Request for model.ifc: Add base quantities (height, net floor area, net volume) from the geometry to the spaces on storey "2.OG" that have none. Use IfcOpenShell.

First a look at what the model holds.

```python
import ifcopenshell
import ifcopenshell.util.element
import ifcopenshell.util.unit

model = ifcopenshell.open("model.ifc")
print(model.schema)
for unit_type in ("LENGTHUNIT", "AREAUNIT", "VOLUMEUNIT"):
    print(unit_type, ifcopenshell.util.unit.calculate_unit_scale(model, unit_type))
storey = next(s for s in model.by_type("IfcBuildingStorey") if s.Name == "2.OG")
spaces = [e for e in ifcopenshell.util.element.get_decomposition(storey) if e.is_a("IfcSpace")]
for e in sorted(spaces, key=lambda e: e.id()):
    print(e.id(), e.is_a(), e.Name, list(ifcopenshell.util.element.get_psets(e, qtos_only=True)), sep=" | ")
```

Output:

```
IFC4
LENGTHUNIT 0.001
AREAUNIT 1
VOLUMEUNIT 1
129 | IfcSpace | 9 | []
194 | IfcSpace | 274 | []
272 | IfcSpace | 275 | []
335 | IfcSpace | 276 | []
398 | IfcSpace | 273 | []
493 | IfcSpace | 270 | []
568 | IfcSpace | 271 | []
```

```python
import ifcopenshell
import ifcopenshell.api.pset
import ifcopenshell.geom
import ifcopenshell.util.element
import ifcopenshell.util.shape
import ifcopenshell.util.unit

model = ifcopenshell.open("model.ifc")
unit_scale = ifcopenshell.util.unit.calculate_unit_scale(model)
area_scale = ifcopenshell.util.unit.calculate_unit_scale(model, "AREAUNIT")
volume_scale = ifcopenshell.util.unit.calculate_unit_scale(model, "VOLUMEUNIT")
settings = ifcopenshell.geom.settings()

storey = next(s for s in model.by_type("IfcBuildingStorey") if s.Name == "2.OG")
spaces = [e for e in ifcopenshell.util.element.get_decomposition(storey) if e.is_a("IfcSpace")]

for e in sorted(spaces, key=lambda e: e.id()):
    if ifcopenshell.util.element.get_psets(e, qtos_only=True, should_inherit=False):
        continue
    # Geometry comes back in metres, in the element's own axes.
    shape = ifcopenshell.geom.create_shape(settings, e)
    values = {
        "Height": ifcopenshell.util.shape.get_z(shape.geometry) / unit_scale,
        "NetFloorArea": ifcopenshell.util.shape.get_footprint_area(shape.geometry) / area_scale,
        "NetVolume": ifcopenshell.util.shape.get_volume(shape.geometry) / volume_scale,
    }
    qto = ifcopenshell.api.pset.add_qto(model, product=e, name="Qto_SpaceBaseQuantities")
    ifcopenshell.api.pset.edit_qto(model, qto=qto, properties=values)
    print(e.id(), {k: round(v, 3) for k, v in values.items()})

model.write("model_rev.ifc")
```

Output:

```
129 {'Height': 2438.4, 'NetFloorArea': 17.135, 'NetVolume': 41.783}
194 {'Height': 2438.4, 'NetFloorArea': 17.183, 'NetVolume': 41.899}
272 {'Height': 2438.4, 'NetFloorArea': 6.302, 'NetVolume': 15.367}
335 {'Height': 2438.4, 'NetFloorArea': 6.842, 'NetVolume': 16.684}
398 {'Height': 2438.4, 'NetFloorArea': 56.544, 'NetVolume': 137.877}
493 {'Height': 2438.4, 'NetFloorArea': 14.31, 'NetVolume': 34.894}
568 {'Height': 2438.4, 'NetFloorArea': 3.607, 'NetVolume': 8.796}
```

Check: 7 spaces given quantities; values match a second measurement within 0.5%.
